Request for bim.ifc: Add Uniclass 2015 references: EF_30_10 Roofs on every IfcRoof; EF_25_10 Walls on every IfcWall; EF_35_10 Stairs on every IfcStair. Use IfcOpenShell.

First a look at what the model holds.

```python
import ifcopenshell

model = ifcopenshell.open("bim.ifc")
print(model.schema)
print("classifications:", [c.Name for c in model.by_type("IfcClassification")])
for ifc_class in ("IfcDoor", "IfcRoof", "IfcStair", "IfcWall", "IfcWindow"):
    print(ifc_class, len(model.by_type(ifc_class)))
```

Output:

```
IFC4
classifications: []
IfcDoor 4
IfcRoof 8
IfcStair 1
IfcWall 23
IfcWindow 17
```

```python
import ifcopenshell
import ifcopenshell.api.classification

model = ifcopenshell.open("bim.ifc")

system = ifcopenshell.api.classification.add_classification(model, classification="Uniclass 2015")

codes = {
    "IfcRoof": ("EF_30_10", "Roofs"),
    "IfcWall": ("EF_25_10", "Walls"),
    "IfcStair": ("EF_35_10", "Stairs"),
}
for ifc_class, (code, name) in codes.items():
    products = model.by_type(ifc_class)
    ifcopenshell.api.classification.add_reference(
        model, products=products, classification=system, identification=code, name=name
    )
    print(code, len(products))

model.write("bim_v2.ifc")
```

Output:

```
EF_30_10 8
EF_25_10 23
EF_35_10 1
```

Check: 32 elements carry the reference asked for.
